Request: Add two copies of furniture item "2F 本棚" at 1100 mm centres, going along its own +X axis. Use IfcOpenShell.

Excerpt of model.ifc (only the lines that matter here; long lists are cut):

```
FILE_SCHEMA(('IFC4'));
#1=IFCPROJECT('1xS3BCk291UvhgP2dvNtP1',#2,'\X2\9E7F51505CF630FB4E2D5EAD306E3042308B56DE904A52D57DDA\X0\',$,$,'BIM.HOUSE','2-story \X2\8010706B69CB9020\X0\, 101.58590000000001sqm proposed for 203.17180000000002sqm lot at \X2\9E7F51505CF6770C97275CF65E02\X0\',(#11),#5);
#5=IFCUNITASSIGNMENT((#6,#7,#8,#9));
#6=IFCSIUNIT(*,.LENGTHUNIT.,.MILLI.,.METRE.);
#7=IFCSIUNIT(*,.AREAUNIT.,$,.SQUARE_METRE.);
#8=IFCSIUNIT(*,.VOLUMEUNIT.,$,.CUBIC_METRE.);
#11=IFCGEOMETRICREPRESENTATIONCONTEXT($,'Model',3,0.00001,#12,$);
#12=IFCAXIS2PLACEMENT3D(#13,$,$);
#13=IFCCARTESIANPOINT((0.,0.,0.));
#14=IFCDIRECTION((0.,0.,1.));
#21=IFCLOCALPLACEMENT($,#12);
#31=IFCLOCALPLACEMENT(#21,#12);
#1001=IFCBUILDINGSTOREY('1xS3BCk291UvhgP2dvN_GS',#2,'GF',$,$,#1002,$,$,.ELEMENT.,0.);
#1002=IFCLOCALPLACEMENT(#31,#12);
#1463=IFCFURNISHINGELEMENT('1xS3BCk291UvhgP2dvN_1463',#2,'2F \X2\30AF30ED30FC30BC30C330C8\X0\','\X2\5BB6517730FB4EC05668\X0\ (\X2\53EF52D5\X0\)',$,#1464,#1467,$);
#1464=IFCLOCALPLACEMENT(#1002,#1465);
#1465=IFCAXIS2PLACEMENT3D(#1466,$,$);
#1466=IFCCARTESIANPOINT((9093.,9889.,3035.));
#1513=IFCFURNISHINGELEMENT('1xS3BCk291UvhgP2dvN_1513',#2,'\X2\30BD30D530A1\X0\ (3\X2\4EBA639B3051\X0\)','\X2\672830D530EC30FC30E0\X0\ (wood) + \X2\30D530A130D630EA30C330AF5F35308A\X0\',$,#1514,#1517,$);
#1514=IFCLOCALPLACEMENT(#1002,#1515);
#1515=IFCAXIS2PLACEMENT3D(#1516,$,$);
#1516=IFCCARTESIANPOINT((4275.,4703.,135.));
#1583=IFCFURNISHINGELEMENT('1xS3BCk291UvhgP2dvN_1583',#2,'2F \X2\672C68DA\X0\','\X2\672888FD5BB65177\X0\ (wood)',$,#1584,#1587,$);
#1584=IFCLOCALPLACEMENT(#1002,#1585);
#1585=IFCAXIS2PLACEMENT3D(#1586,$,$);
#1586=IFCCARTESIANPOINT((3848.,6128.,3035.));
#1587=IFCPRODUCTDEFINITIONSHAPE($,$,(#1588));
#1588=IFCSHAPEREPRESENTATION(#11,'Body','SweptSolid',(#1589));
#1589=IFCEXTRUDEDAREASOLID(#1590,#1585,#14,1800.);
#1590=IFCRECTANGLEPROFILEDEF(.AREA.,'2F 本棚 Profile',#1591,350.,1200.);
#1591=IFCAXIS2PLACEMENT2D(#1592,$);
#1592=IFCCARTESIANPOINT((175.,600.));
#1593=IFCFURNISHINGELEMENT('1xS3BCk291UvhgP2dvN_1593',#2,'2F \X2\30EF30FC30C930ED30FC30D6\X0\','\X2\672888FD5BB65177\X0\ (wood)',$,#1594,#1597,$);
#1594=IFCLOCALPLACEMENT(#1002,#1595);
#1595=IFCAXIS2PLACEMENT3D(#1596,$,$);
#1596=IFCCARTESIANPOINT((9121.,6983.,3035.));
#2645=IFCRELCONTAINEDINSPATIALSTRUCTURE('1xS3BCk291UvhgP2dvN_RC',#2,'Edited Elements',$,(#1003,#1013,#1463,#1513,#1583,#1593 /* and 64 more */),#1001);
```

```python
import ifcopenshell
import ifcopenshell.api.geometry
import ifcopenshell.api.root
import ifcopenshell.util.element
import ifcopenshell.util.placement

model = ifcopenshell.open("model.ifc")


def reuse_history(source, copy):
    """copy_class also copies each property set's owner history, people and application; keep the originals."""
    for rel in copy.IsDefinedBy:
        if rel.is_a("IfcRelDefinesByProperties") and (history := rel.RelatingPropertyDefinition.OwnerHistory):
            rel.RelatingPropertyDefinition.OwnerHistory = source.OwnerHistory
            ifcopenshell.util.element.remove_deep2(model, history)


source = model.by_id(1583)
base = ifcopenshell.util.placement.get_local_placement(source.ObjectPlacement)
step = base[:3, 0] * 1100.0

for i in range(1, 3):
    copy = ifcopenshell.api.root.copy_class(model, product=source)
    copy.Representation = ifcopenshell.util.element.copy_deep(
        model, source.Representation, exclude=["IfcGeometricRepresentationContext", "IfcRepresentationMap"]
    )
    reuse_history(source, copy)
    matrix = base.copy()
    matrix[:3, 3] += i * step
    print("added at", matrix[:3, 3].round(3) + 0.0)
    ifcopenshell.api.geometry.edit_object_placement(model, product=copy, matrix=matrix, is_si=False)

model.write("model_rev.ifc")
```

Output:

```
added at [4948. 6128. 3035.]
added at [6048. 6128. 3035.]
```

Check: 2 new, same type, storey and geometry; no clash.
